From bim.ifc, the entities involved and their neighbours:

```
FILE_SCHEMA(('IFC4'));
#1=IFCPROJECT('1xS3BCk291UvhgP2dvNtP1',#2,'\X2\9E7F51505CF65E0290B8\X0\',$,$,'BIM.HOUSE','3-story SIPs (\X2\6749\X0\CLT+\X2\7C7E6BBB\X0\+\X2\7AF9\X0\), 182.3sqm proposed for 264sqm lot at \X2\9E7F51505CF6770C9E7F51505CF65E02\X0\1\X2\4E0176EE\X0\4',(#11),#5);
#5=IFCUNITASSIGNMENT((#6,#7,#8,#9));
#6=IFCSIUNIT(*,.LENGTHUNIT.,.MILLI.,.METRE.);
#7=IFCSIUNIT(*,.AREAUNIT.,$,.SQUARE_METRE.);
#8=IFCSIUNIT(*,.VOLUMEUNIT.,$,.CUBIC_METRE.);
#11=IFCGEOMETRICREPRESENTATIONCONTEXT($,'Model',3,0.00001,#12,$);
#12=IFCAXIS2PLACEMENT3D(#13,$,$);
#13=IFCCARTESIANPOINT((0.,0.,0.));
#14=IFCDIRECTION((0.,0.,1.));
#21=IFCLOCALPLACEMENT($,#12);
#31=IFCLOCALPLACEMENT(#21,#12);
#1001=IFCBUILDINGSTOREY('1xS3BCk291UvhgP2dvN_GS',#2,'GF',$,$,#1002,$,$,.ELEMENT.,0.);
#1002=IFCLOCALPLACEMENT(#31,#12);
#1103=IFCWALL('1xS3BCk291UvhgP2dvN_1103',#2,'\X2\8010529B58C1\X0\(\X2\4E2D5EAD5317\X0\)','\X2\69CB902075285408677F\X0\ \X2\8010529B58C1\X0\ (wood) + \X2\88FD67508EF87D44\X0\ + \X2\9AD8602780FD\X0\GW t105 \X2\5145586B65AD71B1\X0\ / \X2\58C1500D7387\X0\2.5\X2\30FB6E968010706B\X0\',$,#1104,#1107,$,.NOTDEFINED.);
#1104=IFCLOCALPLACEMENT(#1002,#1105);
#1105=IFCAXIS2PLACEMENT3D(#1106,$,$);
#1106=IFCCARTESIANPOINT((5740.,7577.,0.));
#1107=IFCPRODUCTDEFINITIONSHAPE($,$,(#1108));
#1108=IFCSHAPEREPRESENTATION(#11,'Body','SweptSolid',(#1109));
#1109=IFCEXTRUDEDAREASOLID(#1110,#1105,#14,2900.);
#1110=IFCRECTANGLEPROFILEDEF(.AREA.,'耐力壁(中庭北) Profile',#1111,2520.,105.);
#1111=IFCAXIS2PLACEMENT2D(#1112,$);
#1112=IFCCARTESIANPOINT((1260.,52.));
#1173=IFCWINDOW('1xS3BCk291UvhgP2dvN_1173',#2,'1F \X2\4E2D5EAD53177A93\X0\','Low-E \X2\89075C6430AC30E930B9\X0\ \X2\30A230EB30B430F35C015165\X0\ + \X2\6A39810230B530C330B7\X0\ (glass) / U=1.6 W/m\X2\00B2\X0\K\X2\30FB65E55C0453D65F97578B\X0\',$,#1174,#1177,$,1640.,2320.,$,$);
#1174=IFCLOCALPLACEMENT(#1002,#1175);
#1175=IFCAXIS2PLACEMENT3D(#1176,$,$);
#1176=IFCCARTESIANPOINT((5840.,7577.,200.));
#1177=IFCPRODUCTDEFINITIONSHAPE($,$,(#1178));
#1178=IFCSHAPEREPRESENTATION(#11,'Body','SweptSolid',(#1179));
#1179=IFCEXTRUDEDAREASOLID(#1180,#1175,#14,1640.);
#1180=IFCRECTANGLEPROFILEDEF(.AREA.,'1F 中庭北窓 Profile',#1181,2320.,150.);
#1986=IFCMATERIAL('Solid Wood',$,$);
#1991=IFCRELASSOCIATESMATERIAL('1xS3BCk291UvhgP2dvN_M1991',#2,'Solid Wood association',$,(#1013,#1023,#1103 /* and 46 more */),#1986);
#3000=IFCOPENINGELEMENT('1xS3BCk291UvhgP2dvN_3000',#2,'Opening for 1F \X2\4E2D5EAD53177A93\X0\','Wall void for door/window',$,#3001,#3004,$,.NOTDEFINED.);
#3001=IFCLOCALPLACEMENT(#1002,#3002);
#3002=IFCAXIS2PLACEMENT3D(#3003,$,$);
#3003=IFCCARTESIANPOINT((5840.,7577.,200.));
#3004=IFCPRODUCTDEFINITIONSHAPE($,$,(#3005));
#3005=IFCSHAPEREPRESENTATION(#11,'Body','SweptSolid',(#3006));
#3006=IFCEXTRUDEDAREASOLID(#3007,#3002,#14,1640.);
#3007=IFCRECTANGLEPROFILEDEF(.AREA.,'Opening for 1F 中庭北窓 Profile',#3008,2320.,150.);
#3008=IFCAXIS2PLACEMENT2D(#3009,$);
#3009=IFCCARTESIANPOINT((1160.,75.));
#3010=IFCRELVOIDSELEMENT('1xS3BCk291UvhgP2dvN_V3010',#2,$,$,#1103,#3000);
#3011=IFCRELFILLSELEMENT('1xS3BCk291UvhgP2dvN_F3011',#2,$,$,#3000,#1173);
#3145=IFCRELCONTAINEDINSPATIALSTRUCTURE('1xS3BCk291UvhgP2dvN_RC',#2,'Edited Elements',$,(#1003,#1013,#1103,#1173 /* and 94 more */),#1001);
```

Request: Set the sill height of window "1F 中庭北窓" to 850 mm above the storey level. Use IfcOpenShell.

```python
import numpy as np
import ifcopenshell
import ifcopenshell.api.geometry
import ifcopenshell.geom
import ifcopenshell.util.element
import ifcopenshell.util.placement
import ifcopenshell.util.shape
import ifcopenshell.util.unit

model = ifcopenshell.open("bim.ifc")
unit_scale = ifcopenshell.util.unit.calculate_unit_scale(model)

window = model.by_guid("1xS3BCk291UvhgP2dvN_1173")
opening = window.FillsVoids[0].RelatingOpeningElement
storey = ifcopenshell.util.element.get_container(window, ifc_class="IfcBuildingStorey")
level = ifcopenshell.util.placement.get_local_placement(storey.ObjectPlacement)[2, 3]

# The opening's origin need not be at the sill, so measure its lowest point.
shape = ifcopenshell.geom.create_shape(ifcopenshell.geom.settings(), opening)
bottom = ifcopenshell.util.shape.get_shape_bottom_elevation(shape, shape.geometry) / unit_scale
dz = level + 0.85 / unit_scale - bottom

shift = np.array([0.0, 0.0, dz])
# The window is not placed relative to its opening, so move both.
for product in (opening, window):
    matrix = ifcopenshell.util.placement.get_local_placement(product.ObjectPlacement)
    matrix[:3, 3] += shift
    ifcopenshell.api.geometry.edit_object_placement(model, product=product, matrix=matrix, is_si=False)

print(f"moved by {dz * unit_scale:+.3f} m")

model.write("bim_updated.ifc")
```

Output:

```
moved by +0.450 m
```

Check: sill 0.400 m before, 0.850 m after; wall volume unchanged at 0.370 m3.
